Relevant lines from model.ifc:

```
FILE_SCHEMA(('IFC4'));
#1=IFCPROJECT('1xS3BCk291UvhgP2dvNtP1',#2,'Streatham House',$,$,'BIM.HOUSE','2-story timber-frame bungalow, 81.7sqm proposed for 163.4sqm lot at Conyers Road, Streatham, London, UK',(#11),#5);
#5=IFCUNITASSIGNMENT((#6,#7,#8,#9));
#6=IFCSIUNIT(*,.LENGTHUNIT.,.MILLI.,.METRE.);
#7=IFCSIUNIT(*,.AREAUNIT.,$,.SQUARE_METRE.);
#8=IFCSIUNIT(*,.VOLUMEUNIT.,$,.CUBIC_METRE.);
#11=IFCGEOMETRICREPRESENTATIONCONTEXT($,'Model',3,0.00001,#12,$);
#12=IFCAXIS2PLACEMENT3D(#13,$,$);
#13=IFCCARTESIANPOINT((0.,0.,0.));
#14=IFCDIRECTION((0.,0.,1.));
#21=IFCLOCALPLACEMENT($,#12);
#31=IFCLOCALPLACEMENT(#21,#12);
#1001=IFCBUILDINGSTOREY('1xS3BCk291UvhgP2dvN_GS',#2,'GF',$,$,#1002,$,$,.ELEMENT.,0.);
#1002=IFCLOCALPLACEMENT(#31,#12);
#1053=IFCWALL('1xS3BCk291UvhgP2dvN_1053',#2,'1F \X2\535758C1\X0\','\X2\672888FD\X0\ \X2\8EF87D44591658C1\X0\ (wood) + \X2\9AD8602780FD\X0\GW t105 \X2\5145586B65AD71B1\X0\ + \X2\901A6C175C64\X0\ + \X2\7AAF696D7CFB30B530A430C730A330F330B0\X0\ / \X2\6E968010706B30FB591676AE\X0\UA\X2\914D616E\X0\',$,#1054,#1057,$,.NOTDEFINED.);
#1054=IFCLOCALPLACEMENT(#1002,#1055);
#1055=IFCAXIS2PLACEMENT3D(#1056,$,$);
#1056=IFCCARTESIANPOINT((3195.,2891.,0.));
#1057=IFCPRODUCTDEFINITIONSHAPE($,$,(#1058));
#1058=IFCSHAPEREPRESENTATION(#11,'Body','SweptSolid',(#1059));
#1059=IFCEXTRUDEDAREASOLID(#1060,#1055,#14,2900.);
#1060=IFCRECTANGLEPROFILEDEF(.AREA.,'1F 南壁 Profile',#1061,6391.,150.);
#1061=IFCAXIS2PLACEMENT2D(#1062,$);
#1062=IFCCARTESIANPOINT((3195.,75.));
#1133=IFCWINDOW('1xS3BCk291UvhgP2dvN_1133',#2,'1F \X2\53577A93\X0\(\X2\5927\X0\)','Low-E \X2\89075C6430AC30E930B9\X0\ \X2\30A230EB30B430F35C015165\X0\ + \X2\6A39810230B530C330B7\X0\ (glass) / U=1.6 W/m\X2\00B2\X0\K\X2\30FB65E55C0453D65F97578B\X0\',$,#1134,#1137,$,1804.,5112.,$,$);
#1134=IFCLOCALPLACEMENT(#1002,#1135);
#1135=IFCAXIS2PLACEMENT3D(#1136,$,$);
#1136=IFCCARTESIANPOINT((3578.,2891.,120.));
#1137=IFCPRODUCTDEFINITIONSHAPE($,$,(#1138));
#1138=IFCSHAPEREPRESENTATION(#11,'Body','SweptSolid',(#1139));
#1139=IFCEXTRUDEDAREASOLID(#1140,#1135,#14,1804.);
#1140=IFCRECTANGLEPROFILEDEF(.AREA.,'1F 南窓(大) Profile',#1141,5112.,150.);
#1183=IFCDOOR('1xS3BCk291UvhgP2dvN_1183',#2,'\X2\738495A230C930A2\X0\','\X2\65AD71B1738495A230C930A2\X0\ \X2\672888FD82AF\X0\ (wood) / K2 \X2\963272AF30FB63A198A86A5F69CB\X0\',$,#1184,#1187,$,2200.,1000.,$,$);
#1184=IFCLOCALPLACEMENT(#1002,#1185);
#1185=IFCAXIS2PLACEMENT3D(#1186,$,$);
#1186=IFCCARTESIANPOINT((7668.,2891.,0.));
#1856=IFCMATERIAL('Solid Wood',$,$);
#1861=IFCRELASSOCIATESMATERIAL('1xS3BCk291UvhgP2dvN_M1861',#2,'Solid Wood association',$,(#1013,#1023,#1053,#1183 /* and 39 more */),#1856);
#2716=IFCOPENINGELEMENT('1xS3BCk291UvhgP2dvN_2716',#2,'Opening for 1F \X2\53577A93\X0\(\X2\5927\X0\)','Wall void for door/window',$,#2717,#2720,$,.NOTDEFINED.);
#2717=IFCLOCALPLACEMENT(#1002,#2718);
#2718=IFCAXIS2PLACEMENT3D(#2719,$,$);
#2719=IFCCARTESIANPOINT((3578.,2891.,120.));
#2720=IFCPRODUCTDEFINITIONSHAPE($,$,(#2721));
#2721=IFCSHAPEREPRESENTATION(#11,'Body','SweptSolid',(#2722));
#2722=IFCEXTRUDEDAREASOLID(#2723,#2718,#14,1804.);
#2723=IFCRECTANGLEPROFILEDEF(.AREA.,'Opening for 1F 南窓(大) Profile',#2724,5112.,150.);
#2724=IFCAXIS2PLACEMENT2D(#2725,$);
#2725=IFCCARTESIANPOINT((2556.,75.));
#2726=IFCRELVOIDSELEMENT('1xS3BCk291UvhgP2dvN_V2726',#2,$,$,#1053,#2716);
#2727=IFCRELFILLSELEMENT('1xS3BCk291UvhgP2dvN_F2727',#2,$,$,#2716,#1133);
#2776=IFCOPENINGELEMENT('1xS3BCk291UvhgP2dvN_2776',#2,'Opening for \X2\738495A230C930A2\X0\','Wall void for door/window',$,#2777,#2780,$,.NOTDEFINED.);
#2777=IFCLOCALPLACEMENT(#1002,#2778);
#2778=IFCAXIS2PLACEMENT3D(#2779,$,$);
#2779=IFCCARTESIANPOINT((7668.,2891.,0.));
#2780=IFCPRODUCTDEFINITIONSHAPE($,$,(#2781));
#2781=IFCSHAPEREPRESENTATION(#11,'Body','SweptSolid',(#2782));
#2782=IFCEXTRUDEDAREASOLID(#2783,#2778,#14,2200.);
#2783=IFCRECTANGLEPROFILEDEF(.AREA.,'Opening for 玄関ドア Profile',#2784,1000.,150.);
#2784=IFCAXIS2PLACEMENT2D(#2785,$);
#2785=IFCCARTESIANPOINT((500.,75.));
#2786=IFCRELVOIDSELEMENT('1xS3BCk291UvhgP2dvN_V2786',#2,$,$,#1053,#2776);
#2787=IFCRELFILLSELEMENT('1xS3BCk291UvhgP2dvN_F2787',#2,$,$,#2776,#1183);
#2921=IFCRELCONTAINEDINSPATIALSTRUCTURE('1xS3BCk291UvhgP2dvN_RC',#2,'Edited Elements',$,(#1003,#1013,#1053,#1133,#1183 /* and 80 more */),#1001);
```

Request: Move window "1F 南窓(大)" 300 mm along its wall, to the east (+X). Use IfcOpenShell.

```python
import ifcopenshell
import ifcopenshell.api.geometry
import ifcopenshell.util.placement
import ifcopenshell.util.unit

model = ifcopenshell.open("model.ifc")
unit_scale = ifcopenshell.util.unit.calculate_unit_scale(model)

window = model.by_guid("1xS3BCk291UvhgP2dvN_1133")
opening = window.FillsVoids[0].RelatingOpeningElement
wall = opening.VoidsElements[0].RelatingBuildingElement

wall_matrix = ifcopenshell.util.placement.get_local_placement(wall.ObjectPlacement)
shift = wall_matrix[:3, 0] * 0.3 / unit_scale
before = ifcopenshell.util.placement.get_local_placement(window.ObjectPlacement)[:3, 3].copy()

# The window is not placed relative to its opening, so move both.
for product in (opening, window):
    matrix = ifcopenshell.util.placement.get_local_placement(product.ObjectPlacement)
    matrix[:3, 3] += shift
    ifcopenshell.api.geometry.edit_object_placement(model, product=product, matrix=matrix, is_si=False)

after = ifcopenshell.util.placement.get_local_placement(window.ObjectPlacement)[:3, 3]
print("window moved by", (after - before).round(3) + 0.0)

model.write("model_edited.ifc")
```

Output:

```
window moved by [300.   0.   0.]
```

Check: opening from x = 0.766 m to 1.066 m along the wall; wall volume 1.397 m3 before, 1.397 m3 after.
